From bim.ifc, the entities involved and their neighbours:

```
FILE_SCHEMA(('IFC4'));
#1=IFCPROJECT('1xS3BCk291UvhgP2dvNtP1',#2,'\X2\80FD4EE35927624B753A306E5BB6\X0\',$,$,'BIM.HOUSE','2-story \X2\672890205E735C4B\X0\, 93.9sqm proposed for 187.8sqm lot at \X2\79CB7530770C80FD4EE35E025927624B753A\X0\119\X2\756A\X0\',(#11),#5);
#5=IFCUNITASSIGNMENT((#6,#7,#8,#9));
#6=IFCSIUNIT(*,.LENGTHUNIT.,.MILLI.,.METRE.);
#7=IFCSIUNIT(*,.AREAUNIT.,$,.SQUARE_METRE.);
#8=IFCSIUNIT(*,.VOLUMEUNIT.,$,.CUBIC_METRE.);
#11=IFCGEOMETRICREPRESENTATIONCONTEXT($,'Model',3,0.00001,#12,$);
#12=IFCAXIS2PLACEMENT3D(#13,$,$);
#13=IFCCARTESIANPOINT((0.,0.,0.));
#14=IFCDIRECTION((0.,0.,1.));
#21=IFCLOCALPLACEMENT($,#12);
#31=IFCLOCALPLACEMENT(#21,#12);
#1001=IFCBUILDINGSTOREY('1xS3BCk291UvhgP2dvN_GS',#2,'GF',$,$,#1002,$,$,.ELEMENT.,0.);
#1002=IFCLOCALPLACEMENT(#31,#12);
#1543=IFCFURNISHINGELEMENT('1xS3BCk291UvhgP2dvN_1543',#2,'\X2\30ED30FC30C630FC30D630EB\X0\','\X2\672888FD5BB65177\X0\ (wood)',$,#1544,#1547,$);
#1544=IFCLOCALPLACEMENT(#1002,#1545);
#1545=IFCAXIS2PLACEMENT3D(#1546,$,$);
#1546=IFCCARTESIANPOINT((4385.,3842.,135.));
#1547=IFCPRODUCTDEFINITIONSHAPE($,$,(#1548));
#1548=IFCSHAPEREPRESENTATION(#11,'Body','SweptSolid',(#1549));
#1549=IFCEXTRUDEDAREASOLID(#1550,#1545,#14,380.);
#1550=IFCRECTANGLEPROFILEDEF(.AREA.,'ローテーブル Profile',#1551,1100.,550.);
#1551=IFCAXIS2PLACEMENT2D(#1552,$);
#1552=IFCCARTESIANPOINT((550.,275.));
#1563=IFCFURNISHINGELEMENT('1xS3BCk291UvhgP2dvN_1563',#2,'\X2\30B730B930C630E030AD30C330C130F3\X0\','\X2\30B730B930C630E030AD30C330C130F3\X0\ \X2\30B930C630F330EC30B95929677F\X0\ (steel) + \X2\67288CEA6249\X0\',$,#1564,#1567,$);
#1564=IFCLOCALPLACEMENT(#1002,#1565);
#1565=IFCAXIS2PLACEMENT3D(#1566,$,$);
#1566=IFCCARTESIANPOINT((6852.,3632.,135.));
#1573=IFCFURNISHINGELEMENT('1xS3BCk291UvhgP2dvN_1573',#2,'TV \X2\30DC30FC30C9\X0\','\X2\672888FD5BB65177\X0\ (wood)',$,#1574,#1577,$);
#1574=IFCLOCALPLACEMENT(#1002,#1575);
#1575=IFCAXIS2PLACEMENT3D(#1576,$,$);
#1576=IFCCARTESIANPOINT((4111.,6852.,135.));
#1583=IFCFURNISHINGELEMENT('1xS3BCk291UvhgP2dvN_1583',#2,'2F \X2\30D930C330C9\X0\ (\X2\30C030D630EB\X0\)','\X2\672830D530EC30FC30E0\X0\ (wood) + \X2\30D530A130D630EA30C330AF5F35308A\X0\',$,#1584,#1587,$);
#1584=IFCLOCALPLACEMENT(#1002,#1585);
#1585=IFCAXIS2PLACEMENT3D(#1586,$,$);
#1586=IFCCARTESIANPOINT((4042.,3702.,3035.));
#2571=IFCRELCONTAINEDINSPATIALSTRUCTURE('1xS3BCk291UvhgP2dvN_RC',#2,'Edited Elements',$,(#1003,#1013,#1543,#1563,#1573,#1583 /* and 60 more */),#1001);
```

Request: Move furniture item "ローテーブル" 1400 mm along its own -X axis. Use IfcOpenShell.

```python
import ifcopenshell
import ifcopenshell.api.geometry
import ifcopenshell.util.placement
import ifcopenshell.util.unit

model = ifcopenshell.open("bim.ifc")
unit_scale = ifcopenshell.util.unit.calculate_unit_scale(model)

item = model.by_guid("1xS3BCk291UvhgP2dvN_1543")
matrix = ifcopenshell.util.placement.get_local_placement(item.ObjectPlacement)
matrix[:3, 3] -= matrix[:3, 0] * 1.4 / unit_scale
ifcopenshell.api.geometry.edit_object_placement(model, product=item, matrix=matrix, is_si=False)

print(ifcopenshell.util.placement.get_local_placement(item.ObjectPlacement).round(3) + 0.0)

model.write("bim_edited.ifc")
```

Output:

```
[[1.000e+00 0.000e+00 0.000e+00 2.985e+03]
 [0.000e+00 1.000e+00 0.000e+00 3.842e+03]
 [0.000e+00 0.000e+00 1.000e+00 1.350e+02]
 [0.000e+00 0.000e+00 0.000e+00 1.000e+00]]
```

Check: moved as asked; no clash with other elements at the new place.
